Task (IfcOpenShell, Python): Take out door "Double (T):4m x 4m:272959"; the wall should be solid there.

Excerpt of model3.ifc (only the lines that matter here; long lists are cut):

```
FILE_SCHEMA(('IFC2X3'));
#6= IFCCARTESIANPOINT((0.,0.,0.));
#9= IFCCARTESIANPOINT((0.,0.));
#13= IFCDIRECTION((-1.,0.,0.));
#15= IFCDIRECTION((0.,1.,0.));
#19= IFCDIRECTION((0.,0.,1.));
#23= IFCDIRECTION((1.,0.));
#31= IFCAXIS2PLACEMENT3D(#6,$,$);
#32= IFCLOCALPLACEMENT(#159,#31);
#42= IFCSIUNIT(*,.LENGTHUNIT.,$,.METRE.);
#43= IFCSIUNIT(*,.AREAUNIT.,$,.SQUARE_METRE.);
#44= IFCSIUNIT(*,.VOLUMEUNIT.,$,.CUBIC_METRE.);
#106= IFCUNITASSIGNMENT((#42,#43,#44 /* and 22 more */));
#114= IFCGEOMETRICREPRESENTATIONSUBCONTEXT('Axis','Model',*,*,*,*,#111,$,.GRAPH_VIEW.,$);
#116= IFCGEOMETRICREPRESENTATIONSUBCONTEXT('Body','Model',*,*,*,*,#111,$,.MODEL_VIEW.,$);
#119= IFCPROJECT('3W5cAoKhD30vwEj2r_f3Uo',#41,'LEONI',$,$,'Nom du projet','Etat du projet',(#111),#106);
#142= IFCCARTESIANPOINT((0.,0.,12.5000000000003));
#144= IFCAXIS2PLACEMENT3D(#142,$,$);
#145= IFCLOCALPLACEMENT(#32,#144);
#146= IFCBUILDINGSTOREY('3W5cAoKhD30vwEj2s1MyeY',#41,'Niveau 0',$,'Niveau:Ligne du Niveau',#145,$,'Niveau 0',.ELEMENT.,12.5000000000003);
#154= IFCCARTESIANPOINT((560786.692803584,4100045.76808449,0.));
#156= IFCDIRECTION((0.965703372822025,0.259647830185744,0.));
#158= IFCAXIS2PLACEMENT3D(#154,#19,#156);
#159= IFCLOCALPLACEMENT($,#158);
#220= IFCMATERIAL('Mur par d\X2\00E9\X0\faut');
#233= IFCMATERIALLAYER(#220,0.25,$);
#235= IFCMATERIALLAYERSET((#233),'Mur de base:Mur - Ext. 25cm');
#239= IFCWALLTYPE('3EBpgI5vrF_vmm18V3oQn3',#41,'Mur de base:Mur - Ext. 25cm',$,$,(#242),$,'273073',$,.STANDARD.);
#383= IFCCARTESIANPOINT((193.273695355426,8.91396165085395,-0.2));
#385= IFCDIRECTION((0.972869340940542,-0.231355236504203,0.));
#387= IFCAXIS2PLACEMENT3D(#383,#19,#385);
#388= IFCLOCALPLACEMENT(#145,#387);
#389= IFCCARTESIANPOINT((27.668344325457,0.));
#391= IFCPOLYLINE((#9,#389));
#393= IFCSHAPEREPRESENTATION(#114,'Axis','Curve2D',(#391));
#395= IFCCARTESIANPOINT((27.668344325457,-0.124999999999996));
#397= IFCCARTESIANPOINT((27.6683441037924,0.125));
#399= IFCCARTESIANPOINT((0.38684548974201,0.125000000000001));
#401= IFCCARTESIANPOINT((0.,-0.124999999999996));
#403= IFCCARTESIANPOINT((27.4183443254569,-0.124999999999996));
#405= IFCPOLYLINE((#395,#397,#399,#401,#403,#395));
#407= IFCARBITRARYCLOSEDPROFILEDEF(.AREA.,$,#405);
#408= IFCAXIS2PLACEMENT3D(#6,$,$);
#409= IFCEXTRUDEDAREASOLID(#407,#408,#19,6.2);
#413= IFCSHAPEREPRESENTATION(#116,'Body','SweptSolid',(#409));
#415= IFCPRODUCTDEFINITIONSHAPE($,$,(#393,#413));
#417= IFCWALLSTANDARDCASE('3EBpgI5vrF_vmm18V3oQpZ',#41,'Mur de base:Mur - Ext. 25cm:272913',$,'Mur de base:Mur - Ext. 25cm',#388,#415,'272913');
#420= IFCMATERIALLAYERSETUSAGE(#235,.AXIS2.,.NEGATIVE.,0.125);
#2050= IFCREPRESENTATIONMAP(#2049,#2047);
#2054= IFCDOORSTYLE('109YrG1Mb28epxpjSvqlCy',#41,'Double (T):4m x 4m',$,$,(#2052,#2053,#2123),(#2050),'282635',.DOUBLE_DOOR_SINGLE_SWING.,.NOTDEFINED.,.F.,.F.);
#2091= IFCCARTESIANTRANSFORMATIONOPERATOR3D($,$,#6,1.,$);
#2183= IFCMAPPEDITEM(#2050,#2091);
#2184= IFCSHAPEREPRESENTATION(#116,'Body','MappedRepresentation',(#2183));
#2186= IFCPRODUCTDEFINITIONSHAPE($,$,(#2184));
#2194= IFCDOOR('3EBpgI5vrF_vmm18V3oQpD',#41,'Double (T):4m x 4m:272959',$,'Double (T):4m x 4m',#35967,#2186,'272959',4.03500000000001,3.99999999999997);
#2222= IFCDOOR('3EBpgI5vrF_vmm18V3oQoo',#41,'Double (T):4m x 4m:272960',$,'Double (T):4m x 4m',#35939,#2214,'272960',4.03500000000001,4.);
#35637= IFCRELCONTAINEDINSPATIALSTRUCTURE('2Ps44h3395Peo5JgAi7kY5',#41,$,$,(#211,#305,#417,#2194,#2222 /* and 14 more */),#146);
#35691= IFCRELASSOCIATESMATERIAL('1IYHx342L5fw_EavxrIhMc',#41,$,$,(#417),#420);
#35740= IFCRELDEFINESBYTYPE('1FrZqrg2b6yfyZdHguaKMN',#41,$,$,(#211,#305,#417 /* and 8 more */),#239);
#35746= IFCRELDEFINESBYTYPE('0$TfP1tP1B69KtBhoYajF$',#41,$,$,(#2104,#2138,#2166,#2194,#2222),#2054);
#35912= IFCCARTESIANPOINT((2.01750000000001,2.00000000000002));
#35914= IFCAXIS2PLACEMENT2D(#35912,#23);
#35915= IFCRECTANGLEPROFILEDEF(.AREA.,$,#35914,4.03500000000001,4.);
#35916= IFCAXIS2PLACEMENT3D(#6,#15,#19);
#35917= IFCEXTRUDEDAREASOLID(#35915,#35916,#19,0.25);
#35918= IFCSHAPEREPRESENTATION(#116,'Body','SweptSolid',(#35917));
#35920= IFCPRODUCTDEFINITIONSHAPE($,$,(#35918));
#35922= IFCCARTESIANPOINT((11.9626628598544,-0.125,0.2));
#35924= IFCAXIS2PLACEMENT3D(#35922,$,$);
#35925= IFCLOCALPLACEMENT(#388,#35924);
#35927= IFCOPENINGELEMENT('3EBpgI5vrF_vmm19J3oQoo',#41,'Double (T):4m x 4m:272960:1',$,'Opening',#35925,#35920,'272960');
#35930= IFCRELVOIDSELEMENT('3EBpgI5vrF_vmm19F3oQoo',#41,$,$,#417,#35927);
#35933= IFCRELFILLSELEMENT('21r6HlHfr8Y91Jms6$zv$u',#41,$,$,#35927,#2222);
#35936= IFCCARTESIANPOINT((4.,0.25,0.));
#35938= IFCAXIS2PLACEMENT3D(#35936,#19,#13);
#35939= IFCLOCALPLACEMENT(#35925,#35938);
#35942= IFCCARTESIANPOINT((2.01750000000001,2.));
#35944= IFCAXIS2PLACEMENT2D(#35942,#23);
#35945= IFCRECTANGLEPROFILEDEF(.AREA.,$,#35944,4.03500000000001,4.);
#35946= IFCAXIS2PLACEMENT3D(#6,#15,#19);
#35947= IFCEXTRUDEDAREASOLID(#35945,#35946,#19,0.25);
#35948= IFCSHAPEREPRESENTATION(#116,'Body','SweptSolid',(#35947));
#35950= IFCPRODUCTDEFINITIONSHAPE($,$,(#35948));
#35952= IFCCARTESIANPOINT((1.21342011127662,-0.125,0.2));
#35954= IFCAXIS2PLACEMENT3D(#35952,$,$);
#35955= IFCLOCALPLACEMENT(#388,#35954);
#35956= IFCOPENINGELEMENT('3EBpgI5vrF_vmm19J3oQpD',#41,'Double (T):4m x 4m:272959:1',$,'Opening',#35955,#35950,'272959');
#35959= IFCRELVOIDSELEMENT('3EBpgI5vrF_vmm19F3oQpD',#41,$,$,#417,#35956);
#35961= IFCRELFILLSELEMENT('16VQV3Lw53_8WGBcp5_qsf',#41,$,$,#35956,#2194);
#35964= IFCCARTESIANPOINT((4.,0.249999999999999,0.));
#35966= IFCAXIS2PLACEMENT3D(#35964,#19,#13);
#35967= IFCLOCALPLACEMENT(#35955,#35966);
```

```python
import ifcopenshell
import ifcopenshell.api.feature
import ifcopenshell.api.root
import ifcopenshell.geom
import ifcopenshell.util.shape

model = ifcopenshell.open("model3.ifc")
settings = ifcopenshell.geom.settings()


def volume(element):
    """Net volume in cubic metres, openings subtracted."""
    shape = ifcopenshell.geom.create_shape(settings, element)
    return ifcopenshell.util.shape.get_volume(shape.geometry)


door = model.by_id(2194)
opening = door.FillsVoids[0].RelatingOpeningElement
wall = opening.VoidsElements[0].RelatingBuildingElement
before = volume(wall)

ifcopenshell.api.root.remove_product(model, product=door)
ifcopenshell.api.feature.remove_feature(model, feature=opening)

after = volume(wall)

print(f"wall volume {before:.3f} -> {after:.3f} m3")

model.write("model3_edited.ifc")
```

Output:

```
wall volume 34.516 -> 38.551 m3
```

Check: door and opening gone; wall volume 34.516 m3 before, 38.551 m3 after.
